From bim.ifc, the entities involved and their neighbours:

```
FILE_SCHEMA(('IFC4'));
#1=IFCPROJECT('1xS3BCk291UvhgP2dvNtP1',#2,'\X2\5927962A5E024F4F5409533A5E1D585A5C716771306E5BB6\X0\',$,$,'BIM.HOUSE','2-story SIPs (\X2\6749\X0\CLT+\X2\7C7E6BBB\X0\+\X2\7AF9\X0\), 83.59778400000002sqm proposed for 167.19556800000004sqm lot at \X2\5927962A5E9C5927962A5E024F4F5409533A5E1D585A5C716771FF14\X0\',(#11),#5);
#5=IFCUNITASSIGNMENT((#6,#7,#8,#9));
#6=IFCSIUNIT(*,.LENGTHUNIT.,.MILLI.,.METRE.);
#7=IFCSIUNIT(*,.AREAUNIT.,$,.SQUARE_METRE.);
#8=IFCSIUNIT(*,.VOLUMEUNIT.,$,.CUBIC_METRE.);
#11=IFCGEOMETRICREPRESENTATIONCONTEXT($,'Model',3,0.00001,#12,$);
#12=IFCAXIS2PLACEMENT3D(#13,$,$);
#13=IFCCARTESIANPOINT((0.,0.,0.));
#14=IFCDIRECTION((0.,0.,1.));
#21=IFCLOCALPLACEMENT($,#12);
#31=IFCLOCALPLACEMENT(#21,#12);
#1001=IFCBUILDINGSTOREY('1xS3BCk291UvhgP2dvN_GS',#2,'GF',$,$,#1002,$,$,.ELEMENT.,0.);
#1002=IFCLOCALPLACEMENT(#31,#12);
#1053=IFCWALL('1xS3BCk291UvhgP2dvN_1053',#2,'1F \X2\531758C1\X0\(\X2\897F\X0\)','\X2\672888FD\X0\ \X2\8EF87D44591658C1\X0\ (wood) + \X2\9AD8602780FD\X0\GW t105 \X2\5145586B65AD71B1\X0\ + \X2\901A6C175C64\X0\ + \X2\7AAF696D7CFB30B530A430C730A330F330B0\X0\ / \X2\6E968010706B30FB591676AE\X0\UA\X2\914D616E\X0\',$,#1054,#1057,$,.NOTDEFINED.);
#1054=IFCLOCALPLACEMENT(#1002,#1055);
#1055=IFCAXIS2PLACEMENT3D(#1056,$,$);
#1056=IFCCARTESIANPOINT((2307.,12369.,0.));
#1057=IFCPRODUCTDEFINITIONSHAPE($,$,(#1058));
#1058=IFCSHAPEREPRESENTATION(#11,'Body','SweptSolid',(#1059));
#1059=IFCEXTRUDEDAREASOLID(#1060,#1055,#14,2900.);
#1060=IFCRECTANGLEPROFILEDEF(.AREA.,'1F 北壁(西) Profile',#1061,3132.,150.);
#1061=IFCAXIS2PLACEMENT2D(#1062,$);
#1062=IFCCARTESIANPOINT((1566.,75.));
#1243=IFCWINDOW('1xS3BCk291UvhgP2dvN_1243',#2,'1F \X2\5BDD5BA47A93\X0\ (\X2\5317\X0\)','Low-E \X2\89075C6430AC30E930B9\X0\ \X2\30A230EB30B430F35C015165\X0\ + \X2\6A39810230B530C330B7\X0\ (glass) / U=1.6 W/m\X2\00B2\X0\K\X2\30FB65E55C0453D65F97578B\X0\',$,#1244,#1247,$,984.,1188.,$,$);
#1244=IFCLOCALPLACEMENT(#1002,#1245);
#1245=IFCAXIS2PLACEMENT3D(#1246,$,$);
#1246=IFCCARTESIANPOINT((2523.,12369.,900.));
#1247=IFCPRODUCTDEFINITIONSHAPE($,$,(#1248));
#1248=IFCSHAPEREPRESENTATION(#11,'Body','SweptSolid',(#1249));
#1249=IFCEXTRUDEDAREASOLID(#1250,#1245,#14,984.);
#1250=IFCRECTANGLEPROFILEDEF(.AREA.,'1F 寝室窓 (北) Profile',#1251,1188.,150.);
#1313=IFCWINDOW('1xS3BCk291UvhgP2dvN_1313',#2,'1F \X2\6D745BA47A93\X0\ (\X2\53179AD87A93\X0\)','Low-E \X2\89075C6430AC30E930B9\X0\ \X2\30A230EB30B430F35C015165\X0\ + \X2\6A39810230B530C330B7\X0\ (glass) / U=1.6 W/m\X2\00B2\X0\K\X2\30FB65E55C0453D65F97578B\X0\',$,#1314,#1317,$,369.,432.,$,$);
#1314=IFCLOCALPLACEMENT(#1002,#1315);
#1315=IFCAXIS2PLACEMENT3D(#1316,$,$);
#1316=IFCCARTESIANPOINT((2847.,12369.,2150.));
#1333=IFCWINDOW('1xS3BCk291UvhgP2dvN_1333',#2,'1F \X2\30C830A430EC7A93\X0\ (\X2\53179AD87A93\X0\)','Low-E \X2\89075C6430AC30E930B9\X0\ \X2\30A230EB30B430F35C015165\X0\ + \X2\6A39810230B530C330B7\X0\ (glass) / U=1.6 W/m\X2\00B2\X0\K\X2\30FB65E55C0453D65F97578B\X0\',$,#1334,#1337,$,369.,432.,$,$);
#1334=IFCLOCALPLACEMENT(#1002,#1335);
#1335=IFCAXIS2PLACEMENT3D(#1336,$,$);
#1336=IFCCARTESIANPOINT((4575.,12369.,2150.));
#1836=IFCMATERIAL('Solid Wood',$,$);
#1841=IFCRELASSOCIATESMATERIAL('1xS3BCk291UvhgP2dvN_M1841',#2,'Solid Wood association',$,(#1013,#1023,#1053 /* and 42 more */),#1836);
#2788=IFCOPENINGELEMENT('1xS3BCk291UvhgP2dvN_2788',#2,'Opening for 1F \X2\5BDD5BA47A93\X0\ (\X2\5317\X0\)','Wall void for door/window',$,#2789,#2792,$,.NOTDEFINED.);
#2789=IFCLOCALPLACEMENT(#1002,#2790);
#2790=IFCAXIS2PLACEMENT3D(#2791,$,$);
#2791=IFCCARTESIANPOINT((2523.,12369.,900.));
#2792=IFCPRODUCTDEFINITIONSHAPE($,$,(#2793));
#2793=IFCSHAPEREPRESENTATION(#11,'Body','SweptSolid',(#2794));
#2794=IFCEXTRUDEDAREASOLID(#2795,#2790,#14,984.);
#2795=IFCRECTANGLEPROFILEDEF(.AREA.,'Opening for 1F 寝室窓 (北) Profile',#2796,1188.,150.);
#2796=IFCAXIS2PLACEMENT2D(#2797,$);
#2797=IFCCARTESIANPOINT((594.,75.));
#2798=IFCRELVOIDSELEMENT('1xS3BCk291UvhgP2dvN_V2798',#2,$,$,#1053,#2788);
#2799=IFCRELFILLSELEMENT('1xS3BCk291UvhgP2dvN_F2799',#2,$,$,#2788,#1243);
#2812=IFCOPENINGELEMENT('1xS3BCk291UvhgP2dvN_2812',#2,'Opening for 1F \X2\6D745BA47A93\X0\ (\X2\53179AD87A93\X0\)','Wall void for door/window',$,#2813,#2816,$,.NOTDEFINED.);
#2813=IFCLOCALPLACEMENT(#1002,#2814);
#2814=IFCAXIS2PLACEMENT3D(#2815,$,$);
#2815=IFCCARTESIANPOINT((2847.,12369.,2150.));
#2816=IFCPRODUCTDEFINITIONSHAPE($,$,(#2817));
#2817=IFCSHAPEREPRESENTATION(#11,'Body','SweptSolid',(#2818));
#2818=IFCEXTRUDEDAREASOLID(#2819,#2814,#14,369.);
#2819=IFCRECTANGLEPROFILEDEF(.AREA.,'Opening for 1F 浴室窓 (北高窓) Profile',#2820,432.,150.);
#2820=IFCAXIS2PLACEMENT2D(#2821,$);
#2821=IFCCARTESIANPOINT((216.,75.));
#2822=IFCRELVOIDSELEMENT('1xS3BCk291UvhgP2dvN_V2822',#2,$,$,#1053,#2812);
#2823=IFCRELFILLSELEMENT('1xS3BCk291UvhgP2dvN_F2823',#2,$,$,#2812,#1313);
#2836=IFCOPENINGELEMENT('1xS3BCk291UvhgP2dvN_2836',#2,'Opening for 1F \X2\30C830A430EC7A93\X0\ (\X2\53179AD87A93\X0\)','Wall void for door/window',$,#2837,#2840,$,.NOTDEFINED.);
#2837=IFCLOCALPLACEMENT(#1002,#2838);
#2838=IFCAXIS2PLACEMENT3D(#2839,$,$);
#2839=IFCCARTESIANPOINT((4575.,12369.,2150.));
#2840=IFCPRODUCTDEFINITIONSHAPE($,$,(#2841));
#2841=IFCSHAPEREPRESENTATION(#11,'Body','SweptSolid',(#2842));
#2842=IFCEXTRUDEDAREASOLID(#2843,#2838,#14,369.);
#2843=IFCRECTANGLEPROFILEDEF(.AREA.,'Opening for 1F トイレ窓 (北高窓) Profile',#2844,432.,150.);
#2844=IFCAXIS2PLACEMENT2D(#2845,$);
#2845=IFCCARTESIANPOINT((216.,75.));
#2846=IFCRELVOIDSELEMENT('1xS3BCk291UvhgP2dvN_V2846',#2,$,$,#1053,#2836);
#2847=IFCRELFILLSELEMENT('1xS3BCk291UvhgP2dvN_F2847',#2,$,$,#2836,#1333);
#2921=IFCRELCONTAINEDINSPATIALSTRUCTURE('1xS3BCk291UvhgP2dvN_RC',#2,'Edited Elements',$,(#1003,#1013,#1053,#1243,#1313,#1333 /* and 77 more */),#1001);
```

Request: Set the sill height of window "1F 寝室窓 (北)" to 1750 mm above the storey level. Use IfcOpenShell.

```python
import numpy as np
import ifcopenshell
import ifcopenshell.api.geometry
import ifcopenshell.geom
import ifcopenshell.util.element
import ifcopenshell.util.placement
import ifcopenshell.util.shape
import ifcopenshell.util.unit

model = ifcopenshell.open("bim.ifc")
unit_scale = ifcopenshell.util.unit.calculate_unit_scale(model)

window = model.by_id(1243)
opening = window.FillsVoids[0].RelatingOpeningElement
storey = ifcopenshell.util.element.get_container(window, ifc_class="IfcBuildingStorey")
level = ifcopenshell.util.placement.get_local_placement(storey.ObjectPlacement)[2, 3]

# The opening's origin need not be at the sill, so measure its lowest point.
shape = ifcopenshell.geom.create_shape(ifcopenshell.geom.settings(), opening)
bottom = ifcopenshell.util.shape.get_shape_bottom_elevation(shape, shape.geometry) / unit_scale
dz = level + 1.75 / unit_scale - bottom

shift = np.array([0.0, 0.0, dz])
# The window is not placed relative to its opening, so move both.
for product in (opening, window):
    matrix = ifcopenshell.util.placement.get_local_placement(product.ObjectPlacement)
    matrix[:3, 3] += shift
    ifcopenshell.api.geometry.edit_object_placement(model, product=product, matrix=matrix, is_si=False)

print(f"moved by {dz * unit_scale:+.3f} m")

model.write("bim_updated.ifc")
```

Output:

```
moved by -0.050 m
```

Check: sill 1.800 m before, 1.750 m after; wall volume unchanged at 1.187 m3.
